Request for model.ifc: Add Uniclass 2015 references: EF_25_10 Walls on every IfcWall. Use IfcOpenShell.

First a look at what the model holds.

```python
import ifcopenshell

model = ifcopenshell.open("model.ifc")
print(model.schema)
print("classifications:", [c.Name for c in model.by_type("IfcClassification")])
for ifc_class in ("IfcDoor", "IfcRoof", "IfcStair", "IfcWall", "IfcWindow"):
    print(ifc_class, len(model.by_type(ifc_class)))
```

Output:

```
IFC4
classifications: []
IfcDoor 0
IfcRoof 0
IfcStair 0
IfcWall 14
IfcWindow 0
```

```python
import ifcopenshell
import ifcopenshell.api.classification

model = ifcopenshell.open("model.ifc")

system = ifcopenshell.api.classification.add_classification(model, classification="Uniclass 2015")

codes = {
    "IfcWall": ("EF_25_10", "Walls"),
}
for ifc_class, (code, name) in codes.items():
    products = model.by_type(ifc_class)
    ifcopenshell.api.classification.add_reference(
        model, products=products, classification=system, identification=code, name=name
    )
    print(code, len(products))

model.write("model_edited.ifc")
```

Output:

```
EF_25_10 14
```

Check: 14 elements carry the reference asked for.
